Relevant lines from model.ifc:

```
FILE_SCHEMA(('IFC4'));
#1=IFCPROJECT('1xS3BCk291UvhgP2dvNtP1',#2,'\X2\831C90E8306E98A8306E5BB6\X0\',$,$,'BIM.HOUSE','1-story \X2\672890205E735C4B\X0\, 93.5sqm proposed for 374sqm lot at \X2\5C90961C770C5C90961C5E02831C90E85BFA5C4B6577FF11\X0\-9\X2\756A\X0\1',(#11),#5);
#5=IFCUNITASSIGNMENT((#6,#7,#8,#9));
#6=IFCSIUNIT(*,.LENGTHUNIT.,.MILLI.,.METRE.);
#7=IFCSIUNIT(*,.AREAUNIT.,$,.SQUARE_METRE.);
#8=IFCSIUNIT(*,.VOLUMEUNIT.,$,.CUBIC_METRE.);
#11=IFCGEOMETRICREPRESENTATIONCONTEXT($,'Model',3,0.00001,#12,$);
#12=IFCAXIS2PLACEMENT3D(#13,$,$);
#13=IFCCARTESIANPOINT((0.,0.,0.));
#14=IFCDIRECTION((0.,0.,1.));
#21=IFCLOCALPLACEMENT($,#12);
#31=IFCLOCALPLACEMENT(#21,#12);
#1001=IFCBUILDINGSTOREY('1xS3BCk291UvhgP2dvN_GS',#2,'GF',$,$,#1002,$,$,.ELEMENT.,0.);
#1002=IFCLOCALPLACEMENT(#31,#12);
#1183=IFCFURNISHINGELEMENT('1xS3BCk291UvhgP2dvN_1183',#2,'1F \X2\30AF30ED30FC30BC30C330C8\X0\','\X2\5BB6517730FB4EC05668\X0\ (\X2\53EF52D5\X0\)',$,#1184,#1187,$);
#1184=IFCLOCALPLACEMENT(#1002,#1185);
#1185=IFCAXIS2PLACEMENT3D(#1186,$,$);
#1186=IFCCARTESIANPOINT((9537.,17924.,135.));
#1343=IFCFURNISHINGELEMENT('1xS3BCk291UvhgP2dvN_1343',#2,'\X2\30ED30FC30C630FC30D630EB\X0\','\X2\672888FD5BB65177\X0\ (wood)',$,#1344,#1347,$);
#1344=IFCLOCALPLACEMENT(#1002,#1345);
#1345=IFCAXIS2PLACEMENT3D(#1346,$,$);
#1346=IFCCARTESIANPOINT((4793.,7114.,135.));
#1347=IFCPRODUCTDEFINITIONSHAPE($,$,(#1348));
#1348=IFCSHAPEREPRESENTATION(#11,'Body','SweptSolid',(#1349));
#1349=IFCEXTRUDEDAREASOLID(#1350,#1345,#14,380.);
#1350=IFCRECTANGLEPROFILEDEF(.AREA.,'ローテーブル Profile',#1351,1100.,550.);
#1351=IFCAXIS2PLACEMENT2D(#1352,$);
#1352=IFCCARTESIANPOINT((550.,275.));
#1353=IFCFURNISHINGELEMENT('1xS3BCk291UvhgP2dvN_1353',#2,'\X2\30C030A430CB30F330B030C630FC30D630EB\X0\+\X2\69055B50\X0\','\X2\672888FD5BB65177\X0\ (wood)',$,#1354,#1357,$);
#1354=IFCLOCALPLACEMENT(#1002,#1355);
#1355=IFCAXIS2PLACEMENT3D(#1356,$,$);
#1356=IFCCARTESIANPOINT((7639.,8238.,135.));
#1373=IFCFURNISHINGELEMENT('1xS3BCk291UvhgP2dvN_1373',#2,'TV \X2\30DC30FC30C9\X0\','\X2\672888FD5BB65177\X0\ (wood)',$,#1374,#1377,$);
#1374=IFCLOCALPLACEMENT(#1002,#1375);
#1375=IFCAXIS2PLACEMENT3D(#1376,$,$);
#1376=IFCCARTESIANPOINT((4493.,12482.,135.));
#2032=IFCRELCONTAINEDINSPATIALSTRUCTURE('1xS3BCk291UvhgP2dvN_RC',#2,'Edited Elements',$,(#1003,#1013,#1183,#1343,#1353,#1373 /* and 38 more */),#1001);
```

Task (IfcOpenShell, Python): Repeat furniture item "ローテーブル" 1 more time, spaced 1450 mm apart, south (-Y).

```python
import numpy as np
import ifcopenshell
import ifcopenshell.api.geometry
import ifcopenshell.api.root
import ifcopenshell.util.element
import ifcopenshell.util.placement
import ifcopenshell.util.unit

model = ifcopenshell.open("model.ifc")
unit_scale = ifcopenshell.util.unit.calculate_unit_scale(model)


def reuse_history(source, copy):
    """copy_class also copies each property set's owner history, people and application; keep the originals."""
    for rel in copy.IsDefinedBy:
        if rel.is_a("IfcRelDefinesByProperties") and (history := rel.RelatingPropertyDefinition.OwnerHistory):
            rel.RelatingPropertyDefinition.OwnerHistory = source.OwnerHistory
            ifcopenshell.util.element.remove_deep2(model, history)


source = model.by_id(1343)
base = ifcopenshell.util.placement.get_local_placement(source.ObjectPlacement)
step = np.array([0.0, -1.0, 0.0]) * 1.45 / unit_scale

for i in range(1, 2):
    copy = ifcopenshell.api.root.copy_class(model, product=source)
    copy.Representation = ifcopenshell.util.element.copy_deep(
        model, source.Representation, exclude=["IfcGeometricRepresentationContext", "IfcRepresentationMap"]
    )
    reuse_history(source, copy)
    matrix = base.copy()
    matrix[:3, 3] += i * step
    print("added at", matrix[:3, 3].round(3) + 0.0)
    ifcopenshell.api.geometry.edit_object_placement(model, product=copy, matrix=matrix, is_si=False)

model.write("model_edited.ifc")
```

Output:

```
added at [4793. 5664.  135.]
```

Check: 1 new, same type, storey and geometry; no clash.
